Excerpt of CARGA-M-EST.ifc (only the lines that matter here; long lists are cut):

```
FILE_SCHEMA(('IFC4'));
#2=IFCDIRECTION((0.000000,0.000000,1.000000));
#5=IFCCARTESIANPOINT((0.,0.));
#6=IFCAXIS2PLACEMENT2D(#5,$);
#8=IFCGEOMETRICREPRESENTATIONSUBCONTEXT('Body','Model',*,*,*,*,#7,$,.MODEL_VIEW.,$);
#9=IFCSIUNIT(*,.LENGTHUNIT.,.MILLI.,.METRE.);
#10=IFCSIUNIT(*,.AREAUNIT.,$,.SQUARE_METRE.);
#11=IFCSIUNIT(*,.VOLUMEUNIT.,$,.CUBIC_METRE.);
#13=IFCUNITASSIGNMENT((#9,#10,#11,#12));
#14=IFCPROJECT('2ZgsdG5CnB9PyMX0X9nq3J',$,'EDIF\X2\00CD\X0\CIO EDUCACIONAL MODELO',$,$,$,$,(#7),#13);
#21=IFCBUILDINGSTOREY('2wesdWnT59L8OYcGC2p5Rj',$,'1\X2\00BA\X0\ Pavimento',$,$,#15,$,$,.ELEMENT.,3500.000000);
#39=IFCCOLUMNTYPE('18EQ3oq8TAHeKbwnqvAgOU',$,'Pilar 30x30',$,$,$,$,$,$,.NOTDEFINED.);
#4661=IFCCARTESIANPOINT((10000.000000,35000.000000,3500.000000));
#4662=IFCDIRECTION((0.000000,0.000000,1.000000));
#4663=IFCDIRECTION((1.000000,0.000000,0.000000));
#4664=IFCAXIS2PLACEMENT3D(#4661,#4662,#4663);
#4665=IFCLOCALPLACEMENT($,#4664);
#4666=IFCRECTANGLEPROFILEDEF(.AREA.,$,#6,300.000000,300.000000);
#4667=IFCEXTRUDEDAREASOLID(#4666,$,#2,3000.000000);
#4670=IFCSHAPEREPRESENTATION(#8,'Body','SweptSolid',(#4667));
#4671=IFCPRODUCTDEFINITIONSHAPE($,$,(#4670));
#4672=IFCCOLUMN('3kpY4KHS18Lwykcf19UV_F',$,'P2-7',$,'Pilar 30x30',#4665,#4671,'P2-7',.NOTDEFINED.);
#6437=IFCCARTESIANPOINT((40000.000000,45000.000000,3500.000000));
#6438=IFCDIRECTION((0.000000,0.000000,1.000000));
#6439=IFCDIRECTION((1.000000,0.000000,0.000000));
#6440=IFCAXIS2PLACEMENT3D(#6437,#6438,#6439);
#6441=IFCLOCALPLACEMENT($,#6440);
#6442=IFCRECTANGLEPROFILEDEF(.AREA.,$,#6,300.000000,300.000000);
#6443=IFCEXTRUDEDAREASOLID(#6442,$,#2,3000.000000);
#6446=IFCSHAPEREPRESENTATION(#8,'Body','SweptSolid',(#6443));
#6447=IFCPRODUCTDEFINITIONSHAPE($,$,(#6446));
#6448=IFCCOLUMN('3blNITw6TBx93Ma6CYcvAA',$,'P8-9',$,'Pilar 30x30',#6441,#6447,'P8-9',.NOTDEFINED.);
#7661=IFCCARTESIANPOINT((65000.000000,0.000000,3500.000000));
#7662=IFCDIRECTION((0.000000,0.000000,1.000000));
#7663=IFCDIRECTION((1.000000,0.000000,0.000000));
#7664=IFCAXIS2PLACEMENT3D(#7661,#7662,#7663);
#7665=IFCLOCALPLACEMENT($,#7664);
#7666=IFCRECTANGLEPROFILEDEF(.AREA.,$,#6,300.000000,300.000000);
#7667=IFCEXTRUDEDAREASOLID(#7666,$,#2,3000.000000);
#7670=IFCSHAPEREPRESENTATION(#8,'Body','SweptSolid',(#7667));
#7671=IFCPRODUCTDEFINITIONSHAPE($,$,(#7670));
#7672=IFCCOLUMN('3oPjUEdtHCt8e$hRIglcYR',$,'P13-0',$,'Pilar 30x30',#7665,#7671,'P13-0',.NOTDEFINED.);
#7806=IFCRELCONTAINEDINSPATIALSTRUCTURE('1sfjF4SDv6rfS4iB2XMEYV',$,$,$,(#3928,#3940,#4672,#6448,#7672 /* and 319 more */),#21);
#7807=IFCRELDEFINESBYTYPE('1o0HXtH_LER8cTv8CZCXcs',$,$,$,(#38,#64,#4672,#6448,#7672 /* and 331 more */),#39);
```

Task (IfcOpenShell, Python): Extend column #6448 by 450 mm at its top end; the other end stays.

```python
import ifcopenshell
import ifcopenshell.util.representation
import ifcopenshell.util.unit

model = ifcopenshell.open("CARGA-M-EST.ifc")
unit_scale = ifcopenshell.util.unit.calculate_unit_scale(model)

member = model.by_guid("3blNITw6TBx93Ma6CYcvAA")
change = 0.45 / unit_scale

# The extrusion runs towards the end named, so only its depth changes.
body = ifcopenshell.util.representation.get_representation(member, "Model", "Body")
solid = body.Items[0]
old_length = solid.Depth
solid.Depth += change

print(f"length {old_length:g} -> {solid.Depth:g}")

model.write("CARGA-M-EST_updated.ifc")
```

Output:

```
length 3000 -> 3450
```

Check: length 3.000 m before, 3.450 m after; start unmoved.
